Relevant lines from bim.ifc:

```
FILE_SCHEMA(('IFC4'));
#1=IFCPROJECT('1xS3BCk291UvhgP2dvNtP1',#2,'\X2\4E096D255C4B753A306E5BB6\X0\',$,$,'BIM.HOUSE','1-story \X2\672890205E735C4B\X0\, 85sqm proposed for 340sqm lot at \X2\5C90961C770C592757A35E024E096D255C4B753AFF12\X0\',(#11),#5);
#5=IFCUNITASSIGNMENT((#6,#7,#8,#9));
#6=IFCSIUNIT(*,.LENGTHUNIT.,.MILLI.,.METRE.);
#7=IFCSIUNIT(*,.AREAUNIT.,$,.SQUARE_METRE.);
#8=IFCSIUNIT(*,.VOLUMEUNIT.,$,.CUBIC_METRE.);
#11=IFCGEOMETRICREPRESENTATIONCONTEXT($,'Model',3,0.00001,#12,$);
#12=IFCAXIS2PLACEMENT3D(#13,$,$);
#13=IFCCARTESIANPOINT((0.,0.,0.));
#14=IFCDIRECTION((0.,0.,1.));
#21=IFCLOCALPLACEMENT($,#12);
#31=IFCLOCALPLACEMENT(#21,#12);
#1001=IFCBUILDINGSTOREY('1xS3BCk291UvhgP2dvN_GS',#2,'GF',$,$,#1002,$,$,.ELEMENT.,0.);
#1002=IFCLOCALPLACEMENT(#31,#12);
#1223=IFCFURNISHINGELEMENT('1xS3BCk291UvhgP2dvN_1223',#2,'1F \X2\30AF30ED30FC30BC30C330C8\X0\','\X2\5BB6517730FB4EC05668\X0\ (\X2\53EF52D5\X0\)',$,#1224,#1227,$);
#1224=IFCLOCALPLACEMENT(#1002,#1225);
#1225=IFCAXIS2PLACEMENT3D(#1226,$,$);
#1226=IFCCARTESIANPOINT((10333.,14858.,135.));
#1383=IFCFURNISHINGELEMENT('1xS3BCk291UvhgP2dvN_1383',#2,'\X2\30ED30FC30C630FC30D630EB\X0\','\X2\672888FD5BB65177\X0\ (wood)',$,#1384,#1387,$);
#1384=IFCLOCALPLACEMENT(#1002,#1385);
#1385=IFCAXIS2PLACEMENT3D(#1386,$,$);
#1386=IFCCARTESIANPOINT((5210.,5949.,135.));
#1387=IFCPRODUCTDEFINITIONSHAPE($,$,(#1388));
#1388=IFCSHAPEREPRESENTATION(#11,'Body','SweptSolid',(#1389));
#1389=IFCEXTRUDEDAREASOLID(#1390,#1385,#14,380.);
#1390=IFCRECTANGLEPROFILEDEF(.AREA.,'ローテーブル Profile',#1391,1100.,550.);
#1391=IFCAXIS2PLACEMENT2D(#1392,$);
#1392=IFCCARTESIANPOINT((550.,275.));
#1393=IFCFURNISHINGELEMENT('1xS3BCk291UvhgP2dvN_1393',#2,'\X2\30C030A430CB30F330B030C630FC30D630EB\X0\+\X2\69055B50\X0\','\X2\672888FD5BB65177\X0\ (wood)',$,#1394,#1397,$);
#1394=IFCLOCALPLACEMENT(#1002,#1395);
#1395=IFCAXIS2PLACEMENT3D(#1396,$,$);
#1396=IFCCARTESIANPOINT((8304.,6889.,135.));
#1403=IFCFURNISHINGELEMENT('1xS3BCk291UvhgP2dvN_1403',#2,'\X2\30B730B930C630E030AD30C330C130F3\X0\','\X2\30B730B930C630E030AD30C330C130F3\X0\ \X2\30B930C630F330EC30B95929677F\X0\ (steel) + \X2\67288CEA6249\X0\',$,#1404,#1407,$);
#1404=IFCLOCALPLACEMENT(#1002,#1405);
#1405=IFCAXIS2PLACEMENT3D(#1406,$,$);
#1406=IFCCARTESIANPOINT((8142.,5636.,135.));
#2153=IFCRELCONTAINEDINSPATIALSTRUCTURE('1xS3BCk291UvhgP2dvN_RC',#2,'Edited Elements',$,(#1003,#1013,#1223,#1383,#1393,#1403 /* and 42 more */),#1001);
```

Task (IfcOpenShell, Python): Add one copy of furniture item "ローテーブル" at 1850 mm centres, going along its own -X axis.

```python
import ifcopenshell
import ifcopenshell.api.geometry
import ifcopenshell.api.root
import ifcopenshell.util.element
import ifcopenshell.util.placement
import ifcopenshell.util.unit

model = ifcopenshell.open("bim.ifc")
unit_scale = ifcopenshell.util.unit.calculate_unit_scale(model)


def reuse_history(source, copy):
    """copy_class also copies each property set's owner history, people and application; keep the originals."""
    for rel in copy.IsDefinedBy:
        if rel.is_a("IfcRelDefinesByProperties") and (history := rel.RelatingPropertyDefinition.OwnerHistory):
            rel.RelatingPropertyDefinition.OwnerHistory = source.OwnerHistory
            ifcopenshell.util.element.remove_deep2(model, history)


source = model.by_guid("1xS3BCk291UvhgP2dvN_1383")
base = ifcopenshell.util.placement.get_local_placement(source.ObjectPlacement)
step = -base[:3, 0] * 1.85 / unit_scale

for i in range(1, 2):
    copy = ifcopenshell.api.root.copy_class(model, product=source)
    copy.Representation = ifcopenshell.util.element.copy_deep(
        model, source.Representation, exclude=["IfcGeometricRepresentationContext", "IfcRepresentationMap"]
    )
    reuse_history(source, copy)
    matrix = base.copy()
    matrix[:3, 3] += i * step
    print("added at", matrix[:3, 3].round(3) + 0.0)
    ifcopenshell.api.geometry.edit_object_placement(model, product=copy, matrix=matrix, is_si=False)

model.write("bim_v2.ifc")
```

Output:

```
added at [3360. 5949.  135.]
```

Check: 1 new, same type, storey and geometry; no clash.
